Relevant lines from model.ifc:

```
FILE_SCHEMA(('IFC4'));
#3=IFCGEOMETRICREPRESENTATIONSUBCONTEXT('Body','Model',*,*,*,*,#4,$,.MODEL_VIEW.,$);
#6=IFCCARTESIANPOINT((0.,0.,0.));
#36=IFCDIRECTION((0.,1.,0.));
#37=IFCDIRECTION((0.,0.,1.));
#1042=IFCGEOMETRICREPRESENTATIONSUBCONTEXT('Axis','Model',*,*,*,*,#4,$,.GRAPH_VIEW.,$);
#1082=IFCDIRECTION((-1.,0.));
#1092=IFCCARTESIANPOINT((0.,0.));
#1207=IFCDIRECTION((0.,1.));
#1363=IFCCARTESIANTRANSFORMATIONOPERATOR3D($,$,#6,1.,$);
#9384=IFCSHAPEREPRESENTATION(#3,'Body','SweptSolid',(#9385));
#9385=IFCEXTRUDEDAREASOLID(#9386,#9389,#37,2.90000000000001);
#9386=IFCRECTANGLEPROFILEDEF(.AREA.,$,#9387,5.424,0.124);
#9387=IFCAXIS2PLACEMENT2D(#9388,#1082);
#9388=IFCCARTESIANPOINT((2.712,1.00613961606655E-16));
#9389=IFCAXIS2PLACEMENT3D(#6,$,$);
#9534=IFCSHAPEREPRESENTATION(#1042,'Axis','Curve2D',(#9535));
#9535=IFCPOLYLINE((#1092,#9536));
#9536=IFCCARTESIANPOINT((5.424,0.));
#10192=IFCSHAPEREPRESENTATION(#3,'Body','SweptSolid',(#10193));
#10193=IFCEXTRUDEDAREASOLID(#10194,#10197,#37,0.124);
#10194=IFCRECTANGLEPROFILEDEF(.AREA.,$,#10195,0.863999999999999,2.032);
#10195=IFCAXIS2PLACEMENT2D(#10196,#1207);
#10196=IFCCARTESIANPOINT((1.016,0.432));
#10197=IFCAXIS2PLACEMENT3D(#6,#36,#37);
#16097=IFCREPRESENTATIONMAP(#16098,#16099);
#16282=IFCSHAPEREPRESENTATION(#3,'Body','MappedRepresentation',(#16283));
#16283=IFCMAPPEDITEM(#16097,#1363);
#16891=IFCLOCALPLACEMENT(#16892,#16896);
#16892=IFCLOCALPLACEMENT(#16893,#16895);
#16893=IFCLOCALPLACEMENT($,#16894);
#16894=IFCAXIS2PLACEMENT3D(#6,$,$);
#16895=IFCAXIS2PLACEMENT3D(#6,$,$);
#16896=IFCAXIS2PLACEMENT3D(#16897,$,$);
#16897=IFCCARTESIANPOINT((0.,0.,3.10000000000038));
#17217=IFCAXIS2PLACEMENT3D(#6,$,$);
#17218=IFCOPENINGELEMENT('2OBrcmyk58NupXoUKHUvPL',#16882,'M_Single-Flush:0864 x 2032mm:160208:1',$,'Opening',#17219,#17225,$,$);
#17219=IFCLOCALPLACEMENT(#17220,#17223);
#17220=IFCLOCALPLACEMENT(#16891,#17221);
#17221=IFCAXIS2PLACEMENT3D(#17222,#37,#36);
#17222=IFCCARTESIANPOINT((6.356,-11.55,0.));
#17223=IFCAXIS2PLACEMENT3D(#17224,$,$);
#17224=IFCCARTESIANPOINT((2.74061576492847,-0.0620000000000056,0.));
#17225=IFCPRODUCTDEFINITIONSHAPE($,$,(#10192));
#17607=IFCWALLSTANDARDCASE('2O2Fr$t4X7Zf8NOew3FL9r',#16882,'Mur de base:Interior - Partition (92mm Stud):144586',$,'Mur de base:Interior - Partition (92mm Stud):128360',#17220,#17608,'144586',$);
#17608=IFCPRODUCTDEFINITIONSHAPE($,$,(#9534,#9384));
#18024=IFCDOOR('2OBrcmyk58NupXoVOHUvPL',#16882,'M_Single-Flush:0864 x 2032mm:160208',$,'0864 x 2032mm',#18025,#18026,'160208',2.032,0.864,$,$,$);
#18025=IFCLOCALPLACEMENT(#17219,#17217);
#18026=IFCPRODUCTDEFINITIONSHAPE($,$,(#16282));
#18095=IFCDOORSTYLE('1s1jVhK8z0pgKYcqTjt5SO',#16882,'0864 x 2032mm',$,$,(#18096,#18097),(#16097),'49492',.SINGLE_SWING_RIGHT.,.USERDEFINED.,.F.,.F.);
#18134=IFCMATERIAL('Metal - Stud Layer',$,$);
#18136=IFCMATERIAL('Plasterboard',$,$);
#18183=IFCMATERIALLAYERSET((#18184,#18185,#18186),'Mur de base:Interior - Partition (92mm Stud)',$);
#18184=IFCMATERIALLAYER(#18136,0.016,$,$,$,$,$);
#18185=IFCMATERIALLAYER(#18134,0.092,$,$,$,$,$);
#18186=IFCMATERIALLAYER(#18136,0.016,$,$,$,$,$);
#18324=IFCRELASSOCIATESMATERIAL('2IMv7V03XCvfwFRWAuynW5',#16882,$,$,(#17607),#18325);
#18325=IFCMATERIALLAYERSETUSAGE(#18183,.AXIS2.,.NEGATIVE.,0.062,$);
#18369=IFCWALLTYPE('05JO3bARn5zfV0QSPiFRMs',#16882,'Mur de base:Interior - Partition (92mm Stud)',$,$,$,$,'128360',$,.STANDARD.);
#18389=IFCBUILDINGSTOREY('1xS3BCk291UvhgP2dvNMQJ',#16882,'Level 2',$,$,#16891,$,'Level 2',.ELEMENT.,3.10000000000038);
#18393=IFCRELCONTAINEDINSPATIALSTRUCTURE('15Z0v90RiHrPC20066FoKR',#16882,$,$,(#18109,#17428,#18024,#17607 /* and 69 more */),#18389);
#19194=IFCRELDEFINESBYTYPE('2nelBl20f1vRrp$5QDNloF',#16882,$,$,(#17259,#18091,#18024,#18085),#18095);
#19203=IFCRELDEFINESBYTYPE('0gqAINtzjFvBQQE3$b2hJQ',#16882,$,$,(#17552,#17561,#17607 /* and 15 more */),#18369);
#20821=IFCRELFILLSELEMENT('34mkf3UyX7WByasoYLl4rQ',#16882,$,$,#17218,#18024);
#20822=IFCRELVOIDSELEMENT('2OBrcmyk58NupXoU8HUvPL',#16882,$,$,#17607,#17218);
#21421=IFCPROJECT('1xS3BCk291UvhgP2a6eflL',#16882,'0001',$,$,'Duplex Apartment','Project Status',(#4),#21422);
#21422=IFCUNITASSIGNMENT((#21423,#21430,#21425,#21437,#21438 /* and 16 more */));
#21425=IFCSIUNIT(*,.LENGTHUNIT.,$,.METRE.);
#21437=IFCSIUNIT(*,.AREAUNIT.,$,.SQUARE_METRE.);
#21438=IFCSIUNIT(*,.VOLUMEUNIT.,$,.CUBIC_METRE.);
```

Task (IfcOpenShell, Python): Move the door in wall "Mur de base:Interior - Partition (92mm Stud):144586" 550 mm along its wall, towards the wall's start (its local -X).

```python
import ifcopenshell
import ifcopenshell.api.geometry
import ifcopenshell.util.placement

model = ifcopenshell.open("model.ifc")

door = model.by_guid("2OBrcmyk58NupXoVOHUvPL")
opening = door.FillsVoids[0].RelatingOpeningElement
wall = opening.VoidsElements[0].RelatingBuildingElement

wall_matrix = ifcopenshell.util.placement.get_local_placement(wall.ObjectPlacement)
shift = wall_matrix[:3, 0] * -0.55
before = ifcopenshell.util.placement.get_local_placement(door.ObjectPlacement)[:3, 3].copy()

# The door is placed relative to its opening, so it follows when the opening moves.
matrix = ifcopenshell.util.placement.get_local_placement(opening.ObjectPlacement)
matrix[:3, 3] += shift
ifcopenshell.api.geometry.edit_object_placement(
    model, product=opening, matrix=matrix, is_si=False, should_transform_children=True
)

after = ifcopenshell.util.placement.get_local_placement(door.ObjectPlacement)[:3, 3]
print("door moved by", (after - before).round(3) + 0.0)

model.write("model-out.ifc")
```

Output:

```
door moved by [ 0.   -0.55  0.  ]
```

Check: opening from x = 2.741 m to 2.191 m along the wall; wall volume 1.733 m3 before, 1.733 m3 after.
